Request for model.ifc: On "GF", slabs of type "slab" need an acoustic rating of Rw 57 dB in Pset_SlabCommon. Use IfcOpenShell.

First a look at what the model holds.

```python
import ifcopenshell
import ifcopenshell.util.element

model = ifcopenshell.open("model.ifc")
print(model.schema)
storey = next(s for s in model.by_type("IfcBuildingStorey") if s.Name == "GF")
slabs = [e for e in ifcopenshell.util.element.get_decomposition(storey) if e.is_a("IfcSlab")]
seen = {}
for e in slabs:
    element_type = ifcopenshell.util.element.get_type(e)
    key = (element_type.Name if element_type != e and element_type else None, ifcopenshell.util.element.get_pset(e, "Pset_SlabCommon", "AcousticRating"))
    seen[key] = seen.get(key, 0) + 1
for (name, value), count in sorted(seen.items(), key=str):
    print(count, "x", name, "|", value)
```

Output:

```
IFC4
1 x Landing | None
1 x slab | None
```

```python
import ifcopenshell
import ifcopenshell.api.pset
import ifcopenshell.util.element

model = ifcopenshell.open("model.ifc")

storey = next(s for s in model.by_type("IfcBuildingStorey") if s.Name == "GF")
slabs = [e for e in ifcopenshell.util.element.get_decomposition(storey) if e.is_a("IfcSlab")]

count = 0
for e in slabs:
    element_type = ifcopenshell.util.element.get_type(e)
    if element_type in (None, e) or element_type.Name != "slab":
        continue
    # add_pset returns the element's existing set when there is one.
    pset = ifcopenshell.api.pset.add_pset(model, product=e, name="Pset_SlabCommon")
    ifcopenshell.api.pset.edit_pset(model, pset=pset, properties={"AcousticRating": "Rw 57 dB"})
    count += 1

print(count, "slabs updated")

model.write("model-out.ifc")
```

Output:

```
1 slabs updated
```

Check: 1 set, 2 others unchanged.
